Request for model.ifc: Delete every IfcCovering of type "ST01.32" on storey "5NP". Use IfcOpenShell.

First a look at what the model holds.

```python
import ifcopenshell
import ifcopenshell.util.element

model = ifcopenshell.open("model.ifc")
print(model.schema)
storey = next(s for s in model.by_type("IfcBuildingStorey") if s.Name == "5NP")
coverings = [e for e in ifcopenshell.util.element.get_decomposition(storey) if e.is_a("IfcCovering")]
seen = {}
for e in coverings:
    element_type = ifcopenshell.util.element.get_type(e)
    name = element_type.Name if element_type not in (None, e) else None
    seen[name] = seen.get(name, 0) + 1
for name, count in sorted(seen.items(), key=str):
    print(count, "x", name)
```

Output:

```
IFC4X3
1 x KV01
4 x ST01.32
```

```python
import ifcopenshell
import ifcopenshell.api.root
import ifcopenshell.util.element

model = ifcopenshell.open("model.ifc")

storey = next(s for s in model.by_type("IfcBuildingStorey") if s.Name == "5NP")
coverings = [e for e in ifcopenshell.util.element.get_decomposition(storey) if e.is_a("IfcCovering")]
targets = [e for e in coverings if (t := ifcopenshell.util.element.get_type(e)) not in (None, e) and t.Name == "ST01.32"]

for e in targets:
    ifcopenshell.api.root.remove_product(model, product=e)
print(len(targets), "removed")

model.write("model_v2.ifc")
```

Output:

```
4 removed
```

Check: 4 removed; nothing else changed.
